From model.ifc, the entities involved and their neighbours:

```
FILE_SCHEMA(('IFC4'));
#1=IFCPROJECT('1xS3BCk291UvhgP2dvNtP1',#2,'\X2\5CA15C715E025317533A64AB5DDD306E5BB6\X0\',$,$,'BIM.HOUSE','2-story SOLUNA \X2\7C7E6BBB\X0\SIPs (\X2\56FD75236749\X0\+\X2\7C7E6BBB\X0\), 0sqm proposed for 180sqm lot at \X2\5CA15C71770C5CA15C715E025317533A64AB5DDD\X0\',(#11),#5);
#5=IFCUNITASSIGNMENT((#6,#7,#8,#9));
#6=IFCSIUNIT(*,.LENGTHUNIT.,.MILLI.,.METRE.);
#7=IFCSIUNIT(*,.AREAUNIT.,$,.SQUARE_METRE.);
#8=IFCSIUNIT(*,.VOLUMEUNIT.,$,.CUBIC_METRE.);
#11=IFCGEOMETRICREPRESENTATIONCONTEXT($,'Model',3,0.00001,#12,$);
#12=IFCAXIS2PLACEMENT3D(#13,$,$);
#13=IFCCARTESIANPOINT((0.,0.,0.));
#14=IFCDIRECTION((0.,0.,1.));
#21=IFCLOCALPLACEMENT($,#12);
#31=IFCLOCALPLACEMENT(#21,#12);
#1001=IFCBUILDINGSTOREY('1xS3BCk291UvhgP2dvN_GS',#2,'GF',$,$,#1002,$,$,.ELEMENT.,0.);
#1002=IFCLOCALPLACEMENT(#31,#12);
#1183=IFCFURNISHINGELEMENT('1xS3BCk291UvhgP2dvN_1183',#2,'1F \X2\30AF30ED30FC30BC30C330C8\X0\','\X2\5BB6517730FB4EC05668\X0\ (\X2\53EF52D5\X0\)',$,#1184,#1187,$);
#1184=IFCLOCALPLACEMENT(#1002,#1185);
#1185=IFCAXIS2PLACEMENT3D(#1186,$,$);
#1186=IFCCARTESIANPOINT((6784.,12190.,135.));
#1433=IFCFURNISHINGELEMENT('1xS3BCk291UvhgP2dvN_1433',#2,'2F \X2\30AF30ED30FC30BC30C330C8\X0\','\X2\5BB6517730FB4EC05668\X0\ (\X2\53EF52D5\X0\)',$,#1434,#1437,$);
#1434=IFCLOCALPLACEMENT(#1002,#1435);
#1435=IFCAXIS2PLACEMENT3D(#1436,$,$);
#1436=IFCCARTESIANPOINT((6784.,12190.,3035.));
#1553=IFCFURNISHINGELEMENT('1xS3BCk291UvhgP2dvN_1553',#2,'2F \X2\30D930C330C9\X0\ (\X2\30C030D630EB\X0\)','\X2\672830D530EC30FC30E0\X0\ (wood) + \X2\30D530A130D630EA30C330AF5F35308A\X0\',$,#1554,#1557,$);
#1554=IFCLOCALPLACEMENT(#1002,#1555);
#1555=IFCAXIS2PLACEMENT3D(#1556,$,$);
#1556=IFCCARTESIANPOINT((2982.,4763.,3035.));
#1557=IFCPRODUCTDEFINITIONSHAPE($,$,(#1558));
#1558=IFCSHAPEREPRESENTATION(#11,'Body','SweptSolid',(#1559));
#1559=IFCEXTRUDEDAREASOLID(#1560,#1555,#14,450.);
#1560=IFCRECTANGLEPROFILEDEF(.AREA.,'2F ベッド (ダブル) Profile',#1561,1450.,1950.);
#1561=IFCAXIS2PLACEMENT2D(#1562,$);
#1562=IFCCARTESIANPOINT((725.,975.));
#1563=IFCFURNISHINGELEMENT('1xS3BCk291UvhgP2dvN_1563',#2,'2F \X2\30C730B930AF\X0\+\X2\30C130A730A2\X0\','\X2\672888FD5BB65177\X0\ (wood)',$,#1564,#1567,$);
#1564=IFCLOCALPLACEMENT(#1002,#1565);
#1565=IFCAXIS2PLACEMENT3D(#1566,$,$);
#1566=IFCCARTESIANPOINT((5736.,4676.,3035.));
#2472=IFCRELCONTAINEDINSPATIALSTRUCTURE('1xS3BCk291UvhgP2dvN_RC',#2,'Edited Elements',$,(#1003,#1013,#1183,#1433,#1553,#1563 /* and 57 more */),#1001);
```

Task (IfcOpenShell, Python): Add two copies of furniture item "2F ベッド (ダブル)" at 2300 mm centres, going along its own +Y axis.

```python
import ifcopenshell
import ifcopenshell.api.geometry
import ifcopenshell.api.root
import ifcopenshell.util.element
import ifcopenshell.util.placement
import ifcopenshell.util.unit

model = ifcopenshell.open("model.ifc")
unit_scale = ifcopenshell.util.unit.calculate_unit_scale(model)


def reuse_history(source, copy):
    """copy_class also copies each property set's owner history, people and application; keep the originals."""
    for rel in copy.IsDefinedBy:
        if rel.is_a("IfcRelDefinesByProperties") and (history := rel.RelatingPropertyDefinition.OwnerHistory):
            rel.RelatingPropertyDefinition.OwnerHistory = source.OwnerHistory
            ifcopenshell.util.element.remove_deep2(model, history)


source = model.by_guid("1xS3BCk291UvhgP2dvN_1553")
base = ifcopenshell.util.placement.get_local_placement(source.ObjectPlacement)
step = base[:3, 1] * 2.3 / unit_scale

for i in range(1, 3):
    copy = ifcopenshell.api.root.copy_class(model, product=source)
    copy.Representation = ifcopenshell.util.element.copy_deep(
        model, source.Representation, exclude=["IfcGeometricRepresentationContext", "IfcRepresentationMap"]
    )
    reuse_history(source, copy)
    matrix = base.copy()
    matrix[:3, 3] += i * step
    print("added at", matrix[:3, 3].round(3) + 0.0)
    ifcopenshell.api.geometry.edit_object_placement(model, product=copy, matrix=matrix, is_si=False)

model.write("model_v2.ifc")
```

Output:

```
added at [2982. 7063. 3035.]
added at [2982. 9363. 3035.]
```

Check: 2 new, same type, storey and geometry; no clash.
